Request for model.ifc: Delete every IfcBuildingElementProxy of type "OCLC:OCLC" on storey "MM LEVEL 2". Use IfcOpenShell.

First a look at what the model holds.

```python
import ifcopenshell
import ifcopenshell.util.element

model = ifcopenshell.open("model.ifc")
print(model.schema)
storey = next(s for s in model.by_type("IfcBuildingStorey") if s.Name == "MM LEVEL 2")
proxies = [e for e in ifcopenshell.util.element.get_decomposition(storey) if e.is_a("IfcBuildingElementProxy")]
seen = {}
for e in proxies:
    element_type = ifcopenshell.util.element.get_type(e)
    name = element_type.Name if element_type not in (None, e) else None
    seen[name] = seen.get(name, 0) + 1
for name, count in sorted(seen.items(), key=str):
    print(count, "x", name)
```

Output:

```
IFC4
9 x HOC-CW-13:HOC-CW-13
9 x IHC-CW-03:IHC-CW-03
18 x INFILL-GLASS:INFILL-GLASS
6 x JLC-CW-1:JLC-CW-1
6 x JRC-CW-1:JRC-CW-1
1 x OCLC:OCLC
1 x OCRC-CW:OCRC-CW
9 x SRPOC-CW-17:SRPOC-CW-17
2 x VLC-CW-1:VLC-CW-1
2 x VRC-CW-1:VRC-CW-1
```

```python
import ifcopenshell
import ifcopenshell.api.root
import ifcopenshell.util.element

model = ifcopenshell.open("model.ifc")

storey = next(s for s in model.by_type("IfcBuildingStorey") if s.Name == "MM LEVEL 2")
proxies = [e for e in ifcopenshell.util.element.get_decomposition(storey) if e.is_a("IfcBuildingElementProxy")]
targets = [e for e in proxies if (t := ifcopenshell.util.element.get_type(e)) not in (None, e) and t.Name == "OCLC:OCLC"]

for e in targets:
    ifcopenshell.api.root.remove_product(model, product=e)
print(len(targets), "removed")

model.write("model_rev.ifc")
```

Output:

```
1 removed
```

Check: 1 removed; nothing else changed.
